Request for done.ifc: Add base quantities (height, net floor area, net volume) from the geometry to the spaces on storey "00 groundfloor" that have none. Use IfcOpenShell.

First a look at what the model holds.

```python
import ifcopenshell
import ifcopenshell.util.element
import ifcopenshell.util.unit

model = ifcopenshell.open("done.ifc")
print(model.schema)
for unit_type in ("LENGTHUNIT", "AREAUNIT", "VOLUMEUNIT"):
    print(unit_type, ifcopenshell.util.unit.calculate_unit_scale(model, unit_type))
storey = next(s for s in model.by_type("IfcBuildingStorey") if s.Name == "00 groundfloor")
spaces = [e for e in ifcopenshell.util.element.get_decomposition(storey) if e.is_a("IfcSpace")]
for e in sorted(spaces, key=lambda e: e.id()):
    print(e.id(), e.is_a(), e.Name, list(ifcopenshell.util.element.get_psets(e, qtos_only=True)), sep=" | ")
```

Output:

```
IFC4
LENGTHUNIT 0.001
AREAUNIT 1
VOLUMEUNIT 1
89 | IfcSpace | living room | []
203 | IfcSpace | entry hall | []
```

```python
import ifcopenshell
import ifcopenshell.api.pset
import ifcopenshell.geom
import ifcopenshell.util.element
import ifcopenshell.util.shape
import ifcopenshell.util.unit

model = ifcopenshell.open("done.ifc")
unit_scale = ifcopenshell.util.unit.calculate_unit_scale(model)
area_scale = ifcopenshell.util.unit.calculate_unit_scale(model, "AREAUNIT")
volume_scale = ifcopenshell.util.unit.calculate_unit_scale(model, "VOLUMEUNIT")
settings = ifcopenshell.geom.settings()

storey = next(s for s in model.by_type("IfcBuildingStorey") if s.Name == "00 groundfloor")
spaces = [e for e in ifcopenshell.util.element.get_decomposition(storey) if e.is_a("IfcSpace")]

for e in sorted(spaces, key=lambda e: e.id()):
    if ifcopenshell.util.element.get_psets(e, qtos_only=True, should_inherit=False):
        continue
    # Geometry comes back in metres, in the element's own axes.
    shape = ifcopenshell.geom.create_shape(settings, e)
    values = {
        "Height": ifcopenshell.util.shape.get_z(shape.geometry) / unit_scale,
        "NetFloorArea": ifcopenshell.util.shape.get_footprint_area(shape.geometry) / area_scale,
        "NetVolume": ifcopenshell.util.shape.get_volume(shape.geometry) / volume_scale,
    }
    qto = ifcopenshell.api.pset.add_qto(model, product=e, name="Qto_SpaceBaseQuantities")
    ifcopenshell.api.pset.edit_qto(model, qto=qto, properties=values)
    print(e.id(), {k: round(v, 3) for k, v in values.items()})

model.write("done_edited.ifc")
```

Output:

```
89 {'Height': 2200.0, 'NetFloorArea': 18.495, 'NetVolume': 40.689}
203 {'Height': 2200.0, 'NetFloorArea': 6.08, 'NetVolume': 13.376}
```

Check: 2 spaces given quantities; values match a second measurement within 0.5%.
